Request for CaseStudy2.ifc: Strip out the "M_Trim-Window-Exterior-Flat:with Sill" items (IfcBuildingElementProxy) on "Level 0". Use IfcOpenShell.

First a look at what the model holds.

```python
import ifcopenshell
import ifcopenshell.util.element

model = ifcopenshell.open("CaseStudy2.ifc")
print(model.schema)
storey = next(s for s in model.by_type("IfcBuildingStorey") if s.Name == "Level 0")
proxies = [e for e in ifcopenshell.util.element.get_decomposition(storey) if e.is_a("IfcBuildingElementProxy")]
seen = {}
for e in proxies:
    element_type = ifcopenshell.util.element.get_type(e)
    name = element_type.Name if element_type not in (None, e) else None
    seen[name] = seen.get(name, 0) + 1
for name, count in sorted(seen.items(), key=str):
    print(count, "x", name)
```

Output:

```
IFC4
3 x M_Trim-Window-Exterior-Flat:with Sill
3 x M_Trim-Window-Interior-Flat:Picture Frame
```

```python
import ifcopenshell
import ifcopenshell.api.root
import ifcopenshell.util.element

model = ifcopenshell.open("CaseStudy2.ifc")

storey = next(s for s in model.by_type("IfcBuildingStorey") if s.Name == "Level 0")
proxies = [e for e in ifcopenshell.util.element.get_decomposition(storey) if e.is_a("IfcBuildingElementProxy")]
targets = [e for e in proxies if (t := ifcopenshell.util.element.get_type(e)) not in (None, e) and t.Name == "M_Trim-Window-Exterior-Flat:with Sill"]

for e in targets:
    ifcopenshell.api.root.remove_product(model, product=e)
print(len(targets), "removed")

model.write("CaseStudy2_v2.ifc")
```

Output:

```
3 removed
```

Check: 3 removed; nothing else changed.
